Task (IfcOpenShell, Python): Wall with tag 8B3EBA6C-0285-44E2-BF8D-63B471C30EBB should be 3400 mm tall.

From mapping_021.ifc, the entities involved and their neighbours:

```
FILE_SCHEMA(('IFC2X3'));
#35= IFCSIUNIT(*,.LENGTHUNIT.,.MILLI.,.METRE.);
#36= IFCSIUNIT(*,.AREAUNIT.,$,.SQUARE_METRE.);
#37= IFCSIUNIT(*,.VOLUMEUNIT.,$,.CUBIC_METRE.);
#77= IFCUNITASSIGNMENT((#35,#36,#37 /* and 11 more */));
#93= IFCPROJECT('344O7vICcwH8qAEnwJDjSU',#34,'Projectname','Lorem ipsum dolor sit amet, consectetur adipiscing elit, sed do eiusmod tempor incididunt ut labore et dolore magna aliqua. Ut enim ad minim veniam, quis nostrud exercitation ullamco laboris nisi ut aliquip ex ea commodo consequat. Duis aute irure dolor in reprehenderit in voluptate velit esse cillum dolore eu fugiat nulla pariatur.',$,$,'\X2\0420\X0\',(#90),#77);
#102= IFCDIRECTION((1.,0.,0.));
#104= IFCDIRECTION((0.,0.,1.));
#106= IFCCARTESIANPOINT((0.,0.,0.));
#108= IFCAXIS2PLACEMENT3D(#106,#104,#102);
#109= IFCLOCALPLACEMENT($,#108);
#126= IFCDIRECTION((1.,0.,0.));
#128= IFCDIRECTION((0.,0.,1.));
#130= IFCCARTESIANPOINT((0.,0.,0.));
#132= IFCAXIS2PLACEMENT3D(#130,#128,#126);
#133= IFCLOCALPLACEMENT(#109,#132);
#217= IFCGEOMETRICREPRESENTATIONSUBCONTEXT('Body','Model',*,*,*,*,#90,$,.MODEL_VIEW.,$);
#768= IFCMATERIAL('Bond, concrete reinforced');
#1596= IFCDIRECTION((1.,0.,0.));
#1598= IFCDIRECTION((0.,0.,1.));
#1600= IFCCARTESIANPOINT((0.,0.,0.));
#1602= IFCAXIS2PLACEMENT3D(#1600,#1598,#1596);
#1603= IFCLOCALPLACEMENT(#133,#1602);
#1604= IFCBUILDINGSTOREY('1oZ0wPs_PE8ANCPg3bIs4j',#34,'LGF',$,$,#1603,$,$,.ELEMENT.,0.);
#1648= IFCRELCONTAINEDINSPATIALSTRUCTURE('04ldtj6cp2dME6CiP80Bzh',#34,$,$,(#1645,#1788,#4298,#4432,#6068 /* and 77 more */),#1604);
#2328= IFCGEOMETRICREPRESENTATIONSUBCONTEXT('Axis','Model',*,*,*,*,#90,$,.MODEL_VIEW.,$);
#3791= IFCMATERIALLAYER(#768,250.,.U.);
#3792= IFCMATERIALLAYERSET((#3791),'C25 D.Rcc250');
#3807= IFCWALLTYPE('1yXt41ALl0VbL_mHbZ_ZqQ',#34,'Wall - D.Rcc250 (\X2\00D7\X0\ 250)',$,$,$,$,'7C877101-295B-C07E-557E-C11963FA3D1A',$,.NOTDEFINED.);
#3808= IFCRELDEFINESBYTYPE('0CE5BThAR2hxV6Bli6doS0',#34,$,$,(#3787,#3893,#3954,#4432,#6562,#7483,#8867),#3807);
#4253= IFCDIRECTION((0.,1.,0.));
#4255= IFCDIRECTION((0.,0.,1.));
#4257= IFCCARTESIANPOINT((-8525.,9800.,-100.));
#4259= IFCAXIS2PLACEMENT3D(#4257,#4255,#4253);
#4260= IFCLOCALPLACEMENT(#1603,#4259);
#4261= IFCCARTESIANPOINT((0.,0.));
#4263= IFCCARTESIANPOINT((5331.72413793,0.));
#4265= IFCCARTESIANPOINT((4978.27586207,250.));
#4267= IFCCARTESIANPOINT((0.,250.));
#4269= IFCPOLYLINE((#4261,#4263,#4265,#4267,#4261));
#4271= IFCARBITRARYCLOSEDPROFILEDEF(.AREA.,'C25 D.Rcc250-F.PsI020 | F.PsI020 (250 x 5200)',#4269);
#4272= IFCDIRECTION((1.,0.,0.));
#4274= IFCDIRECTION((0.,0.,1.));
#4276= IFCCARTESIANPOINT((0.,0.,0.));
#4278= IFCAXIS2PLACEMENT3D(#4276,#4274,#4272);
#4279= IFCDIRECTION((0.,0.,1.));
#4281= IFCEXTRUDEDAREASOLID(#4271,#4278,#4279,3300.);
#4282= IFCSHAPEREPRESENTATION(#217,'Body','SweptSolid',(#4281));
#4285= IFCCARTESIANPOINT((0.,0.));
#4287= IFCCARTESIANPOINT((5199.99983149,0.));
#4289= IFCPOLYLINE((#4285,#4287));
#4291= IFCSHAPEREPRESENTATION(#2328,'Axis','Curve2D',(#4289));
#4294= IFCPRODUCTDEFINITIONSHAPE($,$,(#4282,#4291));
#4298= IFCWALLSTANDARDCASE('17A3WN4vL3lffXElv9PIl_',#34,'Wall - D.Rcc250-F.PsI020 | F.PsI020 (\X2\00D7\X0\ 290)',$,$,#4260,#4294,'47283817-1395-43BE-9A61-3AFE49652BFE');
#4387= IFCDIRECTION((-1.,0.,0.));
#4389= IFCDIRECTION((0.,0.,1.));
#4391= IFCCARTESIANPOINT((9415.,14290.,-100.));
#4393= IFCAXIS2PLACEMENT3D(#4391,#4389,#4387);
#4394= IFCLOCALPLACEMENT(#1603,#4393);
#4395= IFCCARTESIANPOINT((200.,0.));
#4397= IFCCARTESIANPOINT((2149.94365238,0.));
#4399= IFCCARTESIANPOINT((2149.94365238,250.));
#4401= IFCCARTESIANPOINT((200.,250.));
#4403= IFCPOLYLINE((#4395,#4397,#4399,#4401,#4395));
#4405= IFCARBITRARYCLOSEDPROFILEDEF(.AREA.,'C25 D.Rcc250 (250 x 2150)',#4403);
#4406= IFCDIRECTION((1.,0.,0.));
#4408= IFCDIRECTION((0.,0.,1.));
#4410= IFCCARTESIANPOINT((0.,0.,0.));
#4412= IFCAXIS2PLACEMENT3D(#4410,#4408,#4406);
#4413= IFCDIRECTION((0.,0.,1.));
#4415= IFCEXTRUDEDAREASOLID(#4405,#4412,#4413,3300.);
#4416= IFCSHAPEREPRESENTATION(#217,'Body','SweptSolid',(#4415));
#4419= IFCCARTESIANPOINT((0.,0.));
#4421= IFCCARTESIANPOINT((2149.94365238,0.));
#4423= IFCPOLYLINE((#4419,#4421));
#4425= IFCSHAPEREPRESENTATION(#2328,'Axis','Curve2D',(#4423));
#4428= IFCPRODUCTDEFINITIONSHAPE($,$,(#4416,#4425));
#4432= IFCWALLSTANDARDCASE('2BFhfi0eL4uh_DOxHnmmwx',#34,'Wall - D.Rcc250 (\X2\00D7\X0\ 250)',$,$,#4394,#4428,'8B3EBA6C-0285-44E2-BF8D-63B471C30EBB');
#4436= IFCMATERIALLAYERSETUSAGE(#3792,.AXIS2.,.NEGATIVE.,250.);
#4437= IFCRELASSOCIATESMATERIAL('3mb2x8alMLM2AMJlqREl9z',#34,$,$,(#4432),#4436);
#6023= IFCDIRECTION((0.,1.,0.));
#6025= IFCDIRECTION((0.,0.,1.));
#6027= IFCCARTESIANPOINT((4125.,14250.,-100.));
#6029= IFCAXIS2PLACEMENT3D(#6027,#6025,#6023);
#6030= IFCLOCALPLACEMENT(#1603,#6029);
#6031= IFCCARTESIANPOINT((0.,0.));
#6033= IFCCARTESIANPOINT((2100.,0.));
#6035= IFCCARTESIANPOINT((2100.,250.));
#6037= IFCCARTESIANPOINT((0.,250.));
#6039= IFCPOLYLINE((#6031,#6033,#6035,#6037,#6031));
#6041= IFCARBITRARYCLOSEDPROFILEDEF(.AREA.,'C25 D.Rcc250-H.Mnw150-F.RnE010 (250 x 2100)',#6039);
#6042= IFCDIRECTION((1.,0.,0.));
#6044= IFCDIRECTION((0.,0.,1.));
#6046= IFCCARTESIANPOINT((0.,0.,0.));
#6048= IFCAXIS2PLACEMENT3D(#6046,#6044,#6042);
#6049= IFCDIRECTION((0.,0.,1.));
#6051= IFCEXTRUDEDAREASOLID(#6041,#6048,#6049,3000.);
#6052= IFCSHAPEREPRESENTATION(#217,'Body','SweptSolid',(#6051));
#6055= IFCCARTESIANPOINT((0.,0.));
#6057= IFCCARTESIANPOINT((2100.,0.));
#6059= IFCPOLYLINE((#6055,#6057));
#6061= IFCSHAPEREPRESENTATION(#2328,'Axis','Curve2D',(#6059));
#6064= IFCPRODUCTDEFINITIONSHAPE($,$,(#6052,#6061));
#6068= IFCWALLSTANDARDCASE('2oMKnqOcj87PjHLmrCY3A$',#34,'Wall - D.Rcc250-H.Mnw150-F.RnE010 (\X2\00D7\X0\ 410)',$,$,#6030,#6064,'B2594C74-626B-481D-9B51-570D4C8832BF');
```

```python
import ifcopenshell
import ifcopenshell.geom
import ifcopenshell.util.representation
import ifcopenshell.util.shape

model = ifcopenshell.open("mapping_021.ifc")
settings = ifcopenshell.geom.settings()


def volume(element):
    """Net volume in cubic metres, openings subtracted."""
    shape = ifcopenshell.geom.create_shape(settings, element)
    return ifcopenshell.util.shape.get_volume(shape.geometry)


wall = model.by_guid("2BFhfi0eL4uh_DOxHnmmwx")
before = volume(wall)

body = ifcopenshell.util.representation.get_representation(wall, "Model", "Body")
solid = body.Items[0]
old_height = solid.Depth
solid.Depth = 3400.0
after = volume(wall)

print(f"height {old_height:g} -> {solid.Depth:g}, volume {before:.3f} -> {after:.3f} m3")

model.write("mapping_021_updated.ifc")
```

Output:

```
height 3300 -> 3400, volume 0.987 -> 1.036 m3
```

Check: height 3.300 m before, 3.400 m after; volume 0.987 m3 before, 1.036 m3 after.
